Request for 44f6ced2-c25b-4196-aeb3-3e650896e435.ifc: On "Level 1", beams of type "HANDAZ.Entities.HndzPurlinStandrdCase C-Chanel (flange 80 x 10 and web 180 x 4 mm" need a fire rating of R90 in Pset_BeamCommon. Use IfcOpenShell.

First a look at what the model holds.

```python
import ifcopenshell
import ifcopenshell.util.element

model = ifcopenshell.open("44f6ced2-c25b-4196-aeb3-3e650896e435.ifc")
print(model.schema)
storey = next(s for s in model.by_type("IfcBuildingStorey") if s.Name == "Level 1")
beams = [e for e in ifcopenshell.util.element.get_decomposition(storey) if e.is_a("IfcBeam")]
seen = {}
for e in beams:
    element_type = ifcopenshell.util.element.get_type(e)
    key = (element_type.Name if element_type != e and element_type else None, ifcopenshell.util.element.get_pset(e, "Pset_BeamCommon", "FireRating"))
    seen[key] = seen.get(key, 0) + 1
for (name, value), count in sorted(seen.items(), key=str):
    print(count, "x", name, "|", value)
```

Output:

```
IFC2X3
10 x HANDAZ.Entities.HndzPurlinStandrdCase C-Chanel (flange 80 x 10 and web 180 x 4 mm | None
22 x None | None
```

```python
import ifcopenshell
import ifcopenshell.api.pset
import ifcopenshell.util.element

model = ifcopenshell.open("44f6ced2-c25b-4196-aeb3-3e650896e435.ifc")

storey = next(s for s in model.by_type("IfcBuildingStorey") if s.Name == "Level 1")
beams = [e for e in ifcopenshell.util.element.get_decomposition(storey) if e.is_a("IfcBeam")]

count = 0
for e in beams:
    element_type = ifcopenshell.util.element.get_type(e)
    if element_type in (None, e) or element_type.Name != "HANDAZ.Entities.HndzPurlinStandrdCase C-Chanel (flange 80 x 10 and web 180 x 4 mm":
        continue
    # add_pset returns the element's existing set when there is one.
    pset = ifcopenshell.api.pset.add_pset(model, product=e, name="Pset_BeamCommon")
    ifcopenshell.api.pset.edit_pset(model, pset=pset, properties={"FireRating": "R90"})
    count += 1

print(count, "beams updated")

model.write("44f6ced2-c25b-4196-aeb3-3e650896e435_v2.ifc")
```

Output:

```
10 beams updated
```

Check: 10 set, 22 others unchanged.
